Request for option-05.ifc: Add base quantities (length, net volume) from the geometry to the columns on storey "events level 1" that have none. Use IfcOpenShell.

First a look at what the model holds.

```python
import ifcopenshell
import ifcopenshell.util.element
import ifcopenshell.util.unit

model = ifcopenshell.open("option-05.ifc")
print(model.schema)
for unit_type in ("LENGTHUNIT", "AREAUNIT", "VOLUMEUNIT"):
    print(unit_type, ifcopenshell.util.unit.calculate_unit_scale(model, unit_type))
storey = next(s for s in model.by_type("IfcBuildingStorey") if s.Name == "events level 1")
columns = [e for e in ifcopenshell.util.element.get_decomposition(storey) if e.is_a("IfcColumn")]
for e in sorted(columns, key=lambda e: e.id()):
    print(e.id(), e.is_a(), e.Name, list(ifcopenshell.util.element.get_psets(e, qtos_only=True)), sep=" | ")
```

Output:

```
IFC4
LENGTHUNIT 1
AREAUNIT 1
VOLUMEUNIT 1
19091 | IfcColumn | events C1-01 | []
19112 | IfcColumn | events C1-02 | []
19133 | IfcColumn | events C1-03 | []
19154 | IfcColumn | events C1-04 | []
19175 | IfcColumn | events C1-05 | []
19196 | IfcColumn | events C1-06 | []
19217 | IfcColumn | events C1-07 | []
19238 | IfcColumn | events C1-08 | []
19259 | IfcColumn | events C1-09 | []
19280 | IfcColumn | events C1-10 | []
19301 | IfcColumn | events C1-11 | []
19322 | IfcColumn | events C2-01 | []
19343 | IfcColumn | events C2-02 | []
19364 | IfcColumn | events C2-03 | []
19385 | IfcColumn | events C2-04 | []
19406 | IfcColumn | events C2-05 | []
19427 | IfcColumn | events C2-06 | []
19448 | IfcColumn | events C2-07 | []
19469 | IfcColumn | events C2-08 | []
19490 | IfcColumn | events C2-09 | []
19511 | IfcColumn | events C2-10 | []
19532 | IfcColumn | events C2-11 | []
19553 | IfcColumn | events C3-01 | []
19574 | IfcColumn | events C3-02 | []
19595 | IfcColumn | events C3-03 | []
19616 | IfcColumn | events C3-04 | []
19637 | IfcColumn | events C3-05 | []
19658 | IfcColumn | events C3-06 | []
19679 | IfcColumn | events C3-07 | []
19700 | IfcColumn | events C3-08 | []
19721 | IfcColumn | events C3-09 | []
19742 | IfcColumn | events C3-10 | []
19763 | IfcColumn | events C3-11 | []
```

```python
import ifcopenshell
import ifcopenshell.api.pset
import ifcopenshell.geom
import ifcopenshell.util.element
import ifcopenshell.util.shape
import ifcopenshell.util.unit

model = ifcopenshell.open("option-05.ifc")
unit_scale = ifcopenshell.util.unit.calculate_unit_scale(model)
volume_scale = ifcopenshell.util.unit.calculate_unit_scale(model, "VOLUMEUNIT")
settings = ifcopenshell.geom.settings()

storey = next(s for s in model.by_type("IfcBuildingStorey") if s.Name == "events level 1")
columns = [e for e in ifcopenshell.util.element.get_decomposition(storey) if e.is_a("IfcColumn")]

for e in sorted(columns, key=lambda e: e.id()):
    if ifcopenshell.util.element.get_psets(e, qtos_only=True, should_inherit=False):
        continue
    # Geometry comes back in metres, in the element's own axes.
    shape = ifcopenshell.geom.create_shape(settings, e)
    values = {
        "Length": ifcopenshell.util.shape.get_z(shape.geometry) / unit_scale,
        "NetVolume": ifcopenshell.util.shape.get_volume(shape.geometry) / volume_scale,
    }
    qto = ifcopenshell.api.pset.add_qto(model, product=e, name="Qto_ColumnBaseQuantities")
    ifcopenshell.api.pset.edit_qto(model, qto=qto, properties=values)
    print(e.id(), {k: round(v, 3) for k, v in values.items()})

model.write("option-05-out.ifc")
```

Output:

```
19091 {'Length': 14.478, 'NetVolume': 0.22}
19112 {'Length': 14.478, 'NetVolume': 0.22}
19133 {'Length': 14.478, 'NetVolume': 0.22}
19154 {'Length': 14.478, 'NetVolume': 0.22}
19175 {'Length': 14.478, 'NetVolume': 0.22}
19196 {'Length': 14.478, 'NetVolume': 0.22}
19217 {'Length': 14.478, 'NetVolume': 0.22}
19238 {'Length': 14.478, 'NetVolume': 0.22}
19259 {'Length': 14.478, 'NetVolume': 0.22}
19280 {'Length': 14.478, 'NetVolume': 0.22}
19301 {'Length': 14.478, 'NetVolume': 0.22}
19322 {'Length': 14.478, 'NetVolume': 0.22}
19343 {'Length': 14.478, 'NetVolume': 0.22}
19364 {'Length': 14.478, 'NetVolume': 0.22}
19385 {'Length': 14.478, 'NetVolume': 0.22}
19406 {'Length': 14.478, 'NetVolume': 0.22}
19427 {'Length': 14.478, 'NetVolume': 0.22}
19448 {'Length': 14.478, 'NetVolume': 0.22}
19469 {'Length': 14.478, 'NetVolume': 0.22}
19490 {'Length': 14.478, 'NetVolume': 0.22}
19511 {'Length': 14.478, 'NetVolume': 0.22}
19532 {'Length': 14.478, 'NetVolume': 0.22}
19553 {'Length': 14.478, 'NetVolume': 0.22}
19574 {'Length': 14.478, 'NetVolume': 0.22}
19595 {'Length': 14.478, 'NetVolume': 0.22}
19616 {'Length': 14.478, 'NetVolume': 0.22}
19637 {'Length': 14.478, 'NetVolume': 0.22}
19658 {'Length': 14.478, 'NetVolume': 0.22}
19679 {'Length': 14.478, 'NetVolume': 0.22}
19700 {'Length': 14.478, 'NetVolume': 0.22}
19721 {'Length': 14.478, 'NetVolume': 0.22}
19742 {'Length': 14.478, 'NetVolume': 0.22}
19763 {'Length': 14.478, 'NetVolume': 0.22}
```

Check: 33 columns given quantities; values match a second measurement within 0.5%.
